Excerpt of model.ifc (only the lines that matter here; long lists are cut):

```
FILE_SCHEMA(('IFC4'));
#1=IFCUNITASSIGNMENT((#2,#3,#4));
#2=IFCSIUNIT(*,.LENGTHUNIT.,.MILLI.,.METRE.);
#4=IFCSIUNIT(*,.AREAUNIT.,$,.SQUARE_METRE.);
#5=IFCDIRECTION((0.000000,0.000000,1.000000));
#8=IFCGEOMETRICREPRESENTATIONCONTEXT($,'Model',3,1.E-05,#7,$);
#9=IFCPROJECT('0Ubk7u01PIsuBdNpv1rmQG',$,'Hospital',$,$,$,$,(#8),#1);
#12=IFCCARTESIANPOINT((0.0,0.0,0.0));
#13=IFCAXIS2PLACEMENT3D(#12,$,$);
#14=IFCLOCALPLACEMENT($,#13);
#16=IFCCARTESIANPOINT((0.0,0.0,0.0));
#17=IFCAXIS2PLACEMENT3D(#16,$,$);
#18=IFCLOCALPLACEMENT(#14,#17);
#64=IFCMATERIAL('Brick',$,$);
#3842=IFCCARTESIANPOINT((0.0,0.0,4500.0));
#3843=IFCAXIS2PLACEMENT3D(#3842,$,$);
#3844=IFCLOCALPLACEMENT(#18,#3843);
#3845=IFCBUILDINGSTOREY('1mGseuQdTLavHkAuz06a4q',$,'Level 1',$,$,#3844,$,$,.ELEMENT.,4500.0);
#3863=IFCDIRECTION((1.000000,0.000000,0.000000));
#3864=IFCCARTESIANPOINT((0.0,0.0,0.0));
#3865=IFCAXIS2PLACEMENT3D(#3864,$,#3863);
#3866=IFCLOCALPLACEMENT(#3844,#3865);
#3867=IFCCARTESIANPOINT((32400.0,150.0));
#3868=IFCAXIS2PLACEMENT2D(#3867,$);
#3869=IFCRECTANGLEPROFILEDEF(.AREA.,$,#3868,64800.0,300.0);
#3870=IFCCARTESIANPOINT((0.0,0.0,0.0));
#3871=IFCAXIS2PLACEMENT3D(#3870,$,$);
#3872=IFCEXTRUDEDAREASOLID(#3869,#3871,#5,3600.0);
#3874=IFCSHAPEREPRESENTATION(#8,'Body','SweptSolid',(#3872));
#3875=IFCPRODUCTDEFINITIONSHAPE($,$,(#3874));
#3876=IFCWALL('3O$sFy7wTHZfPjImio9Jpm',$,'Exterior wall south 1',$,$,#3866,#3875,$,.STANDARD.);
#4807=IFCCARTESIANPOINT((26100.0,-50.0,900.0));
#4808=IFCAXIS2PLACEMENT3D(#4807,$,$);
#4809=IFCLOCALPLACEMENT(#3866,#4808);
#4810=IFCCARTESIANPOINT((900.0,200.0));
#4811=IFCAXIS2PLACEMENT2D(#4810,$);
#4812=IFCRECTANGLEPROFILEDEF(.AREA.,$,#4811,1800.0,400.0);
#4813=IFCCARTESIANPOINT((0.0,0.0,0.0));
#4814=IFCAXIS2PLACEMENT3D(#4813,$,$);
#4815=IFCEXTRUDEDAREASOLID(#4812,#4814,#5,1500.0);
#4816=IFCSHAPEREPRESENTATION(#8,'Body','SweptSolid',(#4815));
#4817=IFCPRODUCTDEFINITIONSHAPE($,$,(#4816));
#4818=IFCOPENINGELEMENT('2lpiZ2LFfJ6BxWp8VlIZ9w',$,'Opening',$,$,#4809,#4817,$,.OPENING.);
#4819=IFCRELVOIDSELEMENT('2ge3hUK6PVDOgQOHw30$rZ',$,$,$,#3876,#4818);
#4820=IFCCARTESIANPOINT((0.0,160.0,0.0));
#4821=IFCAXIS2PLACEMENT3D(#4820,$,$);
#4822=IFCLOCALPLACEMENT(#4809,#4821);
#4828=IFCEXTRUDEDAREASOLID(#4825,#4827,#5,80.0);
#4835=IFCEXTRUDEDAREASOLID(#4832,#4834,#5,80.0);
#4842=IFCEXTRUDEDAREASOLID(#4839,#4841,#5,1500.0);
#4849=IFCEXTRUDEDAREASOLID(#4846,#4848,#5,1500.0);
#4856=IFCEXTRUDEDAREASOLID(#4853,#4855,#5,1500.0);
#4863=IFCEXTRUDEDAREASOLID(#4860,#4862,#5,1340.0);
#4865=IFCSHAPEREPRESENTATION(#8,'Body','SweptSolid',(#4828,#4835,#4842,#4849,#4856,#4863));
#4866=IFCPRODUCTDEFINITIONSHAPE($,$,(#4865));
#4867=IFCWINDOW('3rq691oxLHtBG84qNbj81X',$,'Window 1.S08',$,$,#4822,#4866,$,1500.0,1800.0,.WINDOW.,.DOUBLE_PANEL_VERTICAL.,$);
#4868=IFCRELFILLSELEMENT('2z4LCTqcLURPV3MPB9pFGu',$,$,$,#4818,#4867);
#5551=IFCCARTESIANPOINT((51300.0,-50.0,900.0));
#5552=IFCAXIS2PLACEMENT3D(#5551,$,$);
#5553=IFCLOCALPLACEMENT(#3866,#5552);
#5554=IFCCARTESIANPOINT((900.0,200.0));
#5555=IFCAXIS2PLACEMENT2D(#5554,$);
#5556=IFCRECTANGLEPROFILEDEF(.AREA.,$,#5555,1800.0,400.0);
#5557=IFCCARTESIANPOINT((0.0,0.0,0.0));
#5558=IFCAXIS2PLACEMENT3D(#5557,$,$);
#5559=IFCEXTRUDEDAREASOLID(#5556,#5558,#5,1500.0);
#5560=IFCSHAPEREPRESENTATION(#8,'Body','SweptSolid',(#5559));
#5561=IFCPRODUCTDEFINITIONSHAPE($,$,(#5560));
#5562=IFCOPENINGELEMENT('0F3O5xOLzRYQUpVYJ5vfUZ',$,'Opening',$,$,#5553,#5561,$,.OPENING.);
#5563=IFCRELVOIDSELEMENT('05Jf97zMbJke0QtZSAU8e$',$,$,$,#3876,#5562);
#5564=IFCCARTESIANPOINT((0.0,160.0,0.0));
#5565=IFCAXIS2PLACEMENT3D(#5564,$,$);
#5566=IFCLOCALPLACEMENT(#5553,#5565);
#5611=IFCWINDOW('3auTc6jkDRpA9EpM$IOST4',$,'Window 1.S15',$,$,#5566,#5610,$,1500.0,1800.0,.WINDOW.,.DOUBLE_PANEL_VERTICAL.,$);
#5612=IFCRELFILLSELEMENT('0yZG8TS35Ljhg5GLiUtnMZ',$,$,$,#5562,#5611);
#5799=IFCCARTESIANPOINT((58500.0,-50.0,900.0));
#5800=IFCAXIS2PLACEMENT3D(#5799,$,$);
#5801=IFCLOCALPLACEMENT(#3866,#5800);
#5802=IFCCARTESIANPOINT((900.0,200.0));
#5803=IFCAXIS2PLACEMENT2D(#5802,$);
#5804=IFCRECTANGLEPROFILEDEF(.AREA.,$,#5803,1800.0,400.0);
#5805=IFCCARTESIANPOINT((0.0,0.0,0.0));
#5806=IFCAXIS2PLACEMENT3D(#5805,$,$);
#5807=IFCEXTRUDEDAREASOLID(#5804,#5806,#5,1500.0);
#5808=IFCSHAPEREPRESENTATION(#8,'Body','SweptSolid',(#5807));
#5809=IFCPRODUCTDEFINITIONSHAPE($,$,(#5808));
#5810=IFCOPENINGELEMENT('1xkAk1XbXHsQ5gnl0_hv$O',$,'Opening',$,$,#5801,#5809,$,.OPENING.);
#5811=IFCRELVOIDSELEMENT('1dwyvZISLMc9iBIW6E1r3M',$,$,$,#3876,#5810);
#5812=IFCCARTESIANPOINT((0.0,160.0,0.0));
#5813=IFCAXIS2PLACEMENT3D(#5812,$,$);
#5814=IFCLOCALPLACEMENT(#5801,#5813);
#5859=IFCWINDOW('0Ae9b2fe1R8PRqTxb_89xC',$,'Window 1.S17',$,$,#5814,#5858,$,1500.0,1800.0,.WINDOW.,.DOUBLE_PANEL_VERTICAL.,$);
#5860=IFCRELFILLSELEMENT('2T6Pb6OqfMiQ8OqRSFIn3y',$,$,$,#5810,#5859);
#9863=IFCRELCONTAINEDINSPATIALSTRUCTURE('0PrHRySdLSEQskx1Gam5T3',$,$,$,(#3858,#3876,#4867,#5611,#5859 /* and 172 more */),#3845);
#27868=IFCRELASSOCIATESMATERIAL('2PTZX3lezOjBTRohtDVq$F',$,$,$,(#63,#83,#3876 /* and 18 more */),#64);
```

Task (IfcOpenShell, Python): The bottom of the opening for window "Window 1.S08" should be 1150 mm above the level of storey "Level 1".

```python
import numpy as np
import ifcopenshell
import ifcopenshell.api.geometry
import ifcopenshell.geom
import ifcopenshell.util.element
import ifcopenshell.util.placement
import ifcopenshell.util.shape
import ifcopenshell.util.unit

model = ifcopenshell.open("model.ifc")
unit_scale = ifcopenshell.util.unit.calculate_unit_scale(model)

window = model.by_guid("3rq691oxLHtBG84qNbj81X")
opening = window.FillsVoids[0].RelatingOpeningElement
storey = ifcopenshell.util.element.get_container(window, ifc_class="IfcBuildingStorey")
level = ifcopenshell.util.placement.get_local_placement(storey.ObjectPlacement)[2, 3]

# The opening's origin need not be at the sill, so measure its lowest point.
shape = ifcopenshell.geom.create_shape(ifcopenshell.geom.settings(), opening)
bottom = ifcopenshell.util.shape.get_shape_bottom_elevation(shape, shape.geometry) / unit_scale
dz = level + 1.15 / unit_scale - bottom

shift = np.array([0.0, 0.0, dz])
# The window is placed relative to its opening, so it follows when the opening moves.
matrix = ifcopenshell.util.placement.get_local_placement(opening.ObjectPlacement)
matrix[:3, 3] += shift
ifcopenshell.api.geometry.edit_object_placement(
    model, product=opening, matrix=matrix, is_si=False, should_transform_children=True
)

print(f"moved by {dz * unit_scale:+.3f} m")

model.write("model_v2.ifc")
```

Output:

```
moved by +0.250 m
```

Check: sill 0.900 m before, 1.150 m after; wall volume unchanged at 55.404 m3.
